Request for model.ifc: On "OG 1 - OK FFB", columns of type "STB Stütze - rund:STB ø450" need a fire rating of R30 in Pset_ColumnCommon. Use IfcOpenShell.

First a look at what the model holds.

```python
import ifcopenshell
import ifcopenshell.util.element

model = ifcopenshell.open("model.ifc")
print(model.schema)
storey = next(s for s in model.by_type("IfcBuildingStorey") if s.Name == "OG 1 - OK FFB")
columns = [e for e in ifcopenshell.util.element.get_decomposition(storey) if e.is_a("IfcColumn")]
seen = {}
for e in columns:
    element_type = ifcopenshell.util.element.get_type(e)
    key = (element_type.Name if element_type != e and element_type else None, ifcopenshell.util.element.get_pset(e, "Pset_ColumnCommon", "FireRating"))
    seen[key] = seen.get(key, 0) + 1
for (name, value), count in sorted(seen.items(), key=str):
    print(count, "x", name, "|", value)
```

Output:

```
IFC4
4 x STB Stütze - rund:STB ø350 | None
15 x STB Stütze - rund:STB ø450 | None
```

```python
import ifcopenshell
import ifcopenshell.api.pset
import ifcopenshell.util.element

model = ifcopenshell.open("model.ifc")

storey = next(s for s in model.by_type("IfcBuildingStorey") if s.Name == "OG 1 - OK FFB")
columns = [e for e in ifcopenshell.util.element.get_decomposition(storey) if e.is_a("IfcColumn")]

count = 0
for e in columns:
    element_type = ifcopenshell.util.element.get_type(e)
    if element_type in (None, e) or element_type.Name != "STB Stütze - rund:STB ø450":
        continue
    # add_pset returns the element's existing set when there is one.
    pset = ifcopenshell.api.pset.add_pset(model, product=e, name="Pset_ColumnCommon")
    ifcopenshell.api.pset.edit_pset(model, pset=pset, properties={"FireRating": "R30"})
    count += 1

print(count, "columns updated")

model.write("model-out.ifc")
```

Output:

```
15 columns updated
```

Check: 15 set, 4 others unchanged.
